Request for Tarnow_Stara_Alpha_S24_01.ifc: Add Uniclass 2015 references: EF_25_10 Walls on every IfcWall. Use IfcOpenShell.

First a look at what the model holds.

```python
import ifcopenshell

model = ifcopenshell.open("Tarnow_Stara_Alpha_S24_01.ifc")
print(model.schema)
print("classifications:", [c.Name for c in model.by_type("IfcClassification")])
for ifc_class in ("IfcDoor", "IfcRoof", "IfcStair", "IfcWall", "IfcWindow"):
    print(ifc_class, len(model.by_type(ifc_class)))
```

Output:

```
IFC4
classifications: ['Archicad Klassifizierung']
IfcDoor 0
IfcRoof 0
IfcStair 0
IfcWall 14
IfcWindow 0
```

```python
import ifcopenshell
import ifcopenshell.api.classification

model = ifcopenshell.open("Tarnow_Stara_Alpha_S24_01.ifc")

system = ifcopenshell.api.classification.add_classification(model, classification="Uniclass 2015")

codes = {
    "IfcWall": ("EF_25_10", "Walls"),
}
for ifc_class, (code, name) in codes.items():
    products = model.by_type(ifc_class)
    ifcopenshell.api.classification.add_reference(
        model, products=products, classification=system, identification=code, name=name
    )
    print(code, len(products))

model.write("Tarnow_Stara_Alpha_S24_01_updated.ifc")
```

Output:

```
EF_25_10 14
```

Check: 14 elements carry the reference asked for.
